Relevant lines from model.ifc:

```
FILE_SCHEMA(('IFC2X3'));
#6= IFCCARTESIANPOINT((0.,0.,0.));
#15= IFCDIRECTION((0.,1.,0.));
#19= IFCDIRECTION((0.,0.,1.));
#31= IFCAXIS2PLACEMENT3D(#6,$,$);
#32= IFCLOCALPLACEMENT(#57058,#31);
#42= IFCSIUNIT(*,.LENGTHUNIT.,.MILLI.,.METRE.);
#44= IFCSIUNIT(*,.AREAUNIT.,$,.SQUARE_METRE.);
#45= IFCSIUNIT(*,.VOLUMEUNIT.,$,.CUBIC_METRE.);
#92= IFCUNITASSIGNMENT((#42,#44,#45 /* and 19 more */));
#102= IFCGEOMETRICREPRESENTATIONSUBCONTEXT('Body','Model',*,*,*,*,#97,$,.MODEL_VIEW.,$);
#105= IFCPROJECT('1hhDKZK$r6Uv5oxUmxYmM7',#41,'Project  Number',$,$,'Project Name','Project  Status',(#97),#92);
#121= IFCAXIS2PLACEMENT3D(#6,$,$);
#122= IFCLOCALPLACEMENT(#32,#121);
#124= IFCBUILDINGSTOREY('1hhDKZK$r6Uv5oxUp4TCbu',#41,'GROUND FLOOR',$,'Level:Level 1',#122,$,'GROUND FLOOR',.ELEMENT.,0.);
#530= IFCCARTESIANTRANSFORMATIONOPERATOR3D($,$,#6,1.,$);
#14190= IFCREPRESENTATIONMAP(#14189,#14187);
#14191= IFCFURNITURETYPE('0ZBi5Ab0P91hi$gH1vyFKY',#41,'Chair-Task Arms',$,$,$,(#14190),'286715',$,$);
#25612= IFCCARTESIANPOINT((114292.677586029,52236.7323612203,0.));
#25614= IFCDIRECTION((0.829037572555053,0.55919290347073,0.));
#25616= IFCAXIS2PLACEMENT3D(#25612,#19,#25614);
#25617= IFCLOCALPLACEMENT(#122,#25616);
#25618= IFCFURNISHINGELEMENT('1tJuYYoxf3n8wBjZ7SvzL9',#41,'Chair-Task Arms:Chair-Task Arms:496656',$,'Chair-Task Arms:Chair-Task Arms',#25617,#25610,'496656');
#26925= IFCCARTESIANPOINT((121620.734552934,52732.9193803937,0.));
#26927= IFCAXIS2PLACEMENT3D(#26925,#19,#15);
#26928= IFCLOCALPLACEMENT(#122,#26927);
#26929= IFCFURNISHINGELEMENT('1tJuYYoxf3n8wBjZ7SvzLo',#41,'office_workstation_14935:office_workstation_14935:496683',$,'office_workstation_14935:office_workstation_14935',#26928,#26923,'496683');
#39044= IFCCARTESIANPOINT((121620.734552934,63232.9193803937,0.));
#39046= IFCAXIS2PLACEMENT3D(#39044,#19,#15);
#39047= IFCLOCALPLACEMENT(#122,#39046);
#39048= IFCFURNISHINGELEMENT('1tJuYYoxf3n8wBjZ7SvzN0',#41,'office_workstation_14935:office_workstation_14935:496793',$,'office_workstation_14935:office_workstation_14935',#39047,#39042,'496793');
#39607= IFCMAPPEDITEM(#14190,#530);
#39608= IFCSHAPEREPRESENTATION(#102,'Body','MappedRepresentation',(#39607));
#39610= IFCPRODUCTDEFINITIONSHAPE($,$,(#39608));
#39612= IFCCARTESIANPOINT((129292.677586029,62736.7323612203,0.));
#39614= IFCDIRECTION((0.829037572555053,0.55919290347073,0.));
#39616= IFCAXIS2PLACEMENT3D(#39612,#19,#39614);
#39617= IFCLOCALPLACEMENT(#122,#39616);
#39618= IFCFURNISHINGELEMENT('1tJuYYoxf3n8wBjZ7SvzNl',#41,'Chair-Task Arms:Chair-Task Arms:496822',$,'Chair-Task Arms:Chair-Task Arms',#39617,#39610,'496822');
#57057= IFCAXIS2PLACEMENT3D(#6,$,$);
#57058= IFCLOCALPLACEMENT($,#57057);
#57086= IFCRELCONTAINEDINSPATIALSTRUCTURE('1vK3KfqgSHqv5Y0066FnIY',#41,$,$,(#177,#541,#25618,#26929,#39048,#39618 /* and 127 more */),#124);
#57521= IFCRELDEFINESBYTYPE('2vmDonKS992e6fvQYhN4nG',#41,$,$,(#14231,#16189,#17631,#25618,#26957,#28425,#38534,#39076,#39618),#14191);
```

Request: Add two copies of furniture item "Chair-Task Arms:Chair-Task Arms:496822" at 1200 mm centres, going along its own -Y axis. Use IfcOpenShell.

```python
import ifcopenshell
import ifcopenshell.api.geometry
import ifcopenshell.api.root
import ifcopenshell.util.element
import ifcopenshell.util.placement

model = ifcopenshell.open("model.ifc")


def reuse_history(source, copy):
    """copy_class also copies each property set's owner history, people and application; keep the originals."""
    for rel in copy.IsDefinedBy:
        if rel.is_a("IfcRelDefinesByProperties") and (history := rel.RelatingPropertyDefinition.OwnerHistory):
            rel.RelatingPropertyDefinition.OwnerHistory = source.OwnerHistory
            ifcopenshell.util.element.remove_deep2(model, history)


source = model.by_guid("1tJuYYoxf3n8wBjZ7SvzNl")
base = ifcopenshell.util.placement.get_local_placement(source.ObjectPlacement)
step = -base[:3, 1] * 1200.0

for i in range(1, 3):
    copy = ifcopenshell.api.root.copy_class(model, product=source)
    copy.Representation = ifcopenshell.util.element.copy_deep(
        model, source.Representation, exclude=["IfcGeometricRepresentationContext", "IfcRepresentationMap"]
    )
    copy.Name = "Chair-Task Arms:Chair-Task Arms"
    copy.Tag = None
    reuse_history(source, copy)
    matrix = base.copy()
    matrix[:3, 3] += i * step
    print("added at", matrix[:3, 3].round(3) + 0.0)
    ifcopenshell.api.geometry.edit_object_placement(model, product=copy, matrix=matrix, is_si=False)

model.write("model_updated.ifc")
```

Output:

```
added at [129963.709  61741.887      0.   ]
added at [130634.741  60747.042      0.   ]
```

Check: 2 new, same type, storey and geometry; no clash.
